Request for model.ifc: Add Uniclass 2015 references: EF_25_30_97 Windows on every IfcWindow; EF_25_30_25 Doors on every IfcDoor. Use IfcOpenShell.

First a look at what the model holds.

```python
import ifcopenshell

model = ifcopenshell.open("model.ifc")
print(model.schema)
print("classifications:", [c.Name for c in model.by_type("IfcClassification")])
for ifc_class in ("IfcDoor", "IfcRoof", "IfcStair", "IfcWall", "IfcWindow"):
    print(ifc_class, len(model.by_type(ifc_class)))
```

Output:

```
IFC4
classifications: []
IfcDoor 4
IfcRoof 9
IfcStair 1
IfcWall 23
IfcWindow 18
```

```python
import ifcopenshell
import ifcopenshell.api.classification

model = ifcopenshell.open("model.ifc")

system = ifcopenshell.api.classification.add_classification(model, classification="Uniclass 2015")

codes = {
    "IfcWindow": ("EF_25_30_97", "Windows"),
    "IfcDoor": ("EF_25_30_25", "Doors"),
}
for ifc_class, (code, name) in codes.items():
    products = model.by_type(ifc_class)
    ifcopenshell.api.classification.add_reference(
        model, products=products, classification=system, identification=code, name=name
    )
    print(code, len(products))

model.write("model_updated.ifc")
```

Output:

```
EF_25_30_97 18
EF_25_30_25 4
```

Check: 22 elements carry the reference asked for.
